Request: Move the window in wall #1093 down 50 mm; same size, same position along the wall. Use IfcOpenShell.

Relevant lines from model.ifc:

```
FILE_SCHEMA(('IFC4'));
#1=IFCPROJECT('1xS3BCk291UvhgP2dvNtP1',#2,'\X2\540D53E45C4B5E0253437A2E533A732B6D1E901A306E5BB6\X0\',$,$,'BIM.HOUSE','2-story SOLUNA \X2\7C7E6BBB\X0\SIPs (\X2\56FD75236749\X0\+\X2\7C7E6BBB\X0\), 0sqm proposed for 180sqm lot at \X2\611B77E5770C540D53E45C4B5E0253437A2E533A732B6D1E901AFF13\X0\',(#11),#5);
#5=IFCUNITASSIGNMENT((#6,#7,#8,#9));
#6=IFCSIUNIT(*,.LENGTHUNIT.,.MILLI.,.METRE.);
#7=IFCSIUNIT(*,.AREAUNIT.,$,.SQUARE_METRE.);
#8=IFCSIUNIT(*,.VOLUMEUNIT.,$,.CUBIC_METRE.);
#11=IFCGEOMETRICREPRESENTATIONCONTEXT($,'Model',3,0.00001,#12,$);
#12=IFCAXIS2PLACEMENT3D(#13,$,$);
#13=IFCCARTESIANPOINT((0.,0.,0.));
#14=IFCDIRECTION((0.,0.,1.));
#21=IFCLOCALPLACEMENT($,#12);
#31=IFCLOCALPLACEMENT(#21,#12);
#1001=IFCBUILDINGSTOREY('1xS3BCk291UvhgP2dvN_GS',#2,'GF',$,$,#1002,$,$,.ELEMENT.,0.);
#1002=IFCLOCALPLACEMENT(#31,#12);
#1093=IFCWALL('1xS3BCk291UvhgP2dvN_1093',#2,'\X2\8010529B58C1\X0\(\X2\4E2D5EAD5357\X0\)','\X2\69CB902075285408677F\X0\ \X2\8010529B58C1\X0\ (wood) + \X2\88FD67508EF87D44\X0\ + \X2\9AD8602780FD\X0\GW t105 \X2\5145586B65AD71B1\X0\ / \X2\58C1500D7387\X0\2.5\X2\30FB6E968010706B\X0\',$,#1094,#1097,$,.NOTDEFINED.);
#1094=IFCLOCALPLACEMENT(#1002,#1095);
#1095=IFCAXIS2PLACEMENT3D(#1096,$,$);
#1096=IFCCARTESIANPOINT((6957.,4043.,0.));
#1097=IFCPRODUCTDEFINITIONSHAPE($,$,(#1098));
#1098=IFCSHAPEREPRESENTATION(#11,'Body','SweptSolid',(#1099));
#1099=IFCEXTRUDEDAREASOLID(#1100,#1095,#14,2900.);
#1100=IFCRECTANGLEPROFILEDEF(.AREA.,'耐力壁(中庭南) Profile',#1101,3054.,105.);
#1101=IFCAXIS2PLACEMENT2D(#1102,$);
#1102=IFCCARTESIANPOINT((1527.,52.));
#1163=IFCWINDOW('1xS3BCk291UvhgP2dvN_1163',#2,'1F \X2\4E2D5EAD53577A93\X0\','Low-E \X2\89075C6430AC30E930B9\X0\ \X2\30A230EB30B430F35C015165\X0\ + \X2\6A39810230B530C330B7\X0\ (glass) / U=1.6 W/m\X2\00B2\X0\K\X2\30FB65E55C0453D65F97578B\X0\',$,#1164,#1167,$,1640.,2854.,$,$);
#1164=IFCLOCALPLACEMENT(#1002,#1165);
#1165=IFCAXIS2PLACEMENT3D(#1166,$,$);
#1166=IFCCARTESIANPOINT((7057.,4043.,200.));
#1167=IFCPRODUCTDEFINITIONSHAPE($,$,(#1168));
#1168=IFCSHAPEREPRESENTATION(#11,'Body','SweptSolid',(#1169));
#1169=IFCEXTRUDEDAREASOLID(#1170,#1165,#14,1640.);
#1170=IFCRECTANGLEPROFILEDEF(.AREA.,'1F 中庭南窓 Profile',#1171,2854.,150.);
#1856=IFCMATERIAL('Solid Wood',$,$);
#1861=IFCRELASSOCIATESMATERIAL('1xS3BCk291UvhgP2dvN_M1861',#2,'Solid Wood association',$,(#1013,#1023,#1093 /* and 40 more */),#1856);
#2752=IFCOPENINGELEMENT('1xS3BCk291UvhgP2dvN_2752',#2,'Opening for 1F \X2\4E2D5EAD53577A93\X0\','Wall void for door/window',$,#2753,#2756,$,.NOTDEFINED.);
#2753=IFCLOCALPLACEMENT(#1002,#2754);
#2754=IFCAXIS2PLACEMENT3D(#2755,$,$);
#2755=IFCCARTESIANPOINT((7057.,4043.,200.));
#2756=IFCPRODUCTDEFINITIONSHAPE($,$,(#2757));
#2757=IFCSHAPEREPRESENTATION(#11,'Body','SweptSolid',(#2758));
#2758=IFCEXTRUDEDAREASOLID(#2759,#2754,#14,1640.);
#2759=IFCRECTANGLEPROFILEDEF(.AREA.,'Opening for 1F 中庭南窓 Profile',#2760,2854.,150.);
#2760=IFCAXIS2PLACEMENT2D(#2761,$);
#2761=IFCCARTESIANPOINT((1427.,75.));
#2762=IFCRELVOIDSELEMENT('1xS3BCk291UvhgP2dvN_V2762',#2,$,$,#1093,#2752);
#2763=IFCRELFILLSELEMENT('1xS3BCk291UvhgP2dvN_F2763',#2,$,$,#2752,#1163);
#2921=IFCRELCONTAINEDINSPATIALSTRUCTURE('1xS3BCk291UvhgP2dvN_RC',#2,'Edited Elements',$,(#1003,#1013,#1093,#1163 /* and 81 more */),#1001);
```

```python
import numpy as np
import ifcopenshell
import ifcopenshell.api.geometry
import ifcopenshell.util.placement
import ifcopenshell.util.unit

model = ifcopenshell.open("model.ifc")
unit_scale = ifcopenshell.util.unit.calculate_unit_scale(model)

window = model.by_id(1163)
opening = window.FillsVoids[0].RelatingOpeningElement
dz = -0.05 / unit_scale

shift = np.array([0.0, 0.0, dz])
# The window is not placed relative to its opening, so move both.
for product in (opening, window):
    matrix = ifcopenshell.util.placement.get_local_placement(product.ObjectPlacement)
    matrix[:3, 3] += shift
    ifcopenshell.api.geometry.edit_object_placement(model, product=product, matrix=matrix, is_si=False)

print(f"moved by {dz * unit_scale:+.3f} m")

model.write("model_updated.ifc")
```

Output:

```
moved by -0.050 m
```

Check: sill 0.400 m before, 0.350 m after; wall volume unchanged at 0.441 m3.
